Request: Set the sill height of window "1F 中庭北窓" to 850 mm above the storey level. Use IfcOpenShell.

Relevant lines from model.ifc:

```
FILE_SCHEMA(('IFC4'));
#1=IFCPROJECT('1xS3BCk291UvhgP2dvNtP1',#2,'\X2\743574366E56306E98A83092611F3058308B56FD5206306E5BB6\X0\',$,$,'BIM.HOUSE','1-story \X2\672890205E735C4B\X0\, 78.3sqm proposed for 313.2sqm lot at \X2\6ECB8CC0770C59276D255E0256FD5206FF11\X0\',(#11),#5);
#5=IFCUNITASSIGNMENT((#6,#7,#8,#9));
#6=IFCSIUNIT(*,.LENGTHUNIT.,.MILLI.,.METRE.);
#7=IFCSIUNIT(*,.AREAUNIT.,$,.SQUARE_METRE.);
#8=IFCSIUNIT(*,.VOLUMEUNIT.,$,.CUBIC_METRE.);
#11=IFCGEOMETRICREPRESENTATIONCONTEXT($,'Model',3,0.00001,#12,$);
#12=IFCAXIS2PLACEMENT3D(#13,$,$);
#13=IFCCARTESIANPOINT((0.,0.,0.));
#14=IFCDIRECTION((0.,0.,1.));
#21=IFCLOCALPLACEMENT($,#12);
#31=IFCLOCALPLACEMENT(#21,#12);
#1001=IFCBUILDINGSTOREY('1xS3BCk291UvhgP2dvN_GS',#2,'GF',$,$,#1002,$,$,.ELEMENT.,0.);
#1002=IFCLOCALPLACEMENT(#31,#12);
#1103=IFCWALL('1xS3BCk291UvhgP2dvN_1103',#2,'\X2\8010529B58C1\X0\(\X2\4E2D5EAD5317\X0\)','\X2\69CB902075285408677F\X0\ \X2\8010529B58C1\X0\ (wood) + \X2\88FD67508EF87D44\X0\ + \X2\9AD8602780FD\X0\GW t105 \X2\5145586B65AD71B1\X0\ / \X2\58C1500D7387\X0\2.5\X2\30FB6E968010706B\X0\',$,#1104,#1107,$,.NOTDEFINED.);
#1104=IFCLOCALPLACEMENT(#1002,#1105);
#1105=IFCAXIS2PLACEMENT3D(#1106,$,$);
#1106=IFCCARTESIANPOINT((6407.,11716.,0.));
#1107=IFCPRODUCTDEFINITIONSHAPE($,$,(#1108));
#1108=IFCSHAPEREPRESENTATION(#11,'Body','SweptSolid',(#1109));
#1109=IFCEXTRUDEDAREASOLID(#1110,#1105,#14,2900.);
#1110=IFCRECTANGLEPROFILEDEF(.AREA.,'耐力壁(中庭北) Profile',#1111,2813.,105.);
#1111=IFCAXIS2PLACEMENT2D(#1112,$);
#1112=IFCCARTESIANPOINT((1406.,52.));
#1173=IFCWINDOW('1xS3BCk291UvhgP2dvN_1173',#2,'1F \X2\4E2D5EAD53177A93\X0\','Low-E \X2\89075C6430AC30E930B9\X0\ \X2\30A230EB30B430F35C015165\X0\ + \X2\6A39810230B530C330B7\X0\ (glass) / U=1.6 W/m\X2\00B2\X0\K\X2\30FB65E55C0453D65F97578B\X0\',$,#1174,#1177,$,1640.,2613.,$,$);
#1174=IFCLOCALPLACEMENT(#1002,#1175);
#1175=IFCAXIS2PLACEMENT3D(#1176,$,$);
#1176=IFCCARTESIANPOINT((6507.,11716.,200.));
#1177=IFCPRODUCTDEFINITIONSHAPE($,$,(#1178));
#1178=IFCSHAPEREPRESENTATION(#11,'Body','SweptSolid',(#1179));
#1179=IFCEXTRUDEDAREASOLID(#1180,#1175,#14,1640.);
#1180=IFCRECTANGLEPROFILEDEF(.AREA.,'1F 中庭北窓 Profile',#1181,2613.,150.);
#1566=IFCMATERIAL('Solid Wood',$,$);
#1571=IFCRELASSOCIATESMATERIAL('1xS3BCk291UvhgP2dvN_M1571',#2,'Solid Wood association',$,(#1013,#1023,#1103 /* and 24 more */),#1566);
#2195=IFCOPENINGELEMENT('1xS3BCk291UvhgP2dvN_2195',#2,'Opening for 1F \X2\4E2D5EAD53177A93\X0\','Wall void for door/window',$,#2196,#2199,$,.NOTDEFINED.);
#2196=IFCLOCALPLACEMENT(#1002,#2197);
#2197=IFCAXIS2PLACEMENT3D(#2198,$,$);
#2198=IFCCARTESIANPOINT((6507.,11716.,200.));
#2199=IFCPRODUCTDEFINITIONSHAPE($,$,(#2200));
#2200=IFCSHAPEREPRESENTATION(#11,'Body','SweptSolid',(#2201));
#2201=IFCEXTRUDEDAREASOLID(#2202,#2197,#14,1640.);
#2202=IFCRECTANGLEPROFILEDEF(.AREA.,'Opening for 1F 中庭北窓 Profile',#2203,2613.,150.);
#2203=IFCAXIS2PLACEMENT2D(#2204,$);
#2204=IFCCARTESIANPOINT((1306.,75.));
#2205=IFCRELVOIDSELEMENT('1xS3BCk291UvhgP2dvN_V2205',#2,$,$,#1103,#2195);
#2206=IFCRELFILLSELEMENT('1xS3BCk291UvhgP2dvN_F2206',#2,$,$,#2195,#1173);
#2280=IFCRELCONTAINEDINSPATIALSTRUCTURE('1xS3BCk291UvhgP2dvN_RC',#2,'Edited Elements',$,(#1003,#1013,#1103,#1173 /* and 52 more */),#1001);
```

```python
import numpy as np
import ifcopenshell
import ifcopenshell.api.geometry
import ifcopenshell.geom
import ifcopenshell.util.element
import ifcopenshell.util.placement
import ifcopenshell.util.shape
import ifcopenshell.util.unit

model = ifcopenshell.open("model.ifc")
unit_scale = ifcopenshell.util.unit.calculate_unit_scale(model)

window = model.by_guid("1xS3BCk291UvhgP2dvN_1173")
opening = window.FillsVoids[0].RelatingOpeningElement
storey = ifcopenshell.util.element.get_container(window, ifc_class="IfcBuildingStorey")
level = ifcopenshell.util.placement.get_local_placement(storey.ObjectPlacement)[2, 3]

# The opening's origin need not be at the sill, so measure its lowest point.
shape = ifcopenshell.geom.create_shape(ifcopenshell.geom.settings(), opening)
bottom = ifcopenshell.util.shape.get_shape_bottom_elevation(shape, shape.geometry) / unit_scale
dz = level + 0.85 / unit_scale - bottom

shift = np.array([0.0, 0.0, dz])
# The window is not placed relative to its opening, so move both.
for product in (opening, window):
    matrix = ifcopenshell.util.placement.get_local_placement(product.ObjectPlacement)
    matrix[:3, 3] += shift
    ifcopenshell.api.geometry.edit_object_placement(model, product=product, matrix=matrix, is_si=False)

print(f"moved by {dz * unit_scale:+.3f} m")

model.write("model_edited.ifc")
```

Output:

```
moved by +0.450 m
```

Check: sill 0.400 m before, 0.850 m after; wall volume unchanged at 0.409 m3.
